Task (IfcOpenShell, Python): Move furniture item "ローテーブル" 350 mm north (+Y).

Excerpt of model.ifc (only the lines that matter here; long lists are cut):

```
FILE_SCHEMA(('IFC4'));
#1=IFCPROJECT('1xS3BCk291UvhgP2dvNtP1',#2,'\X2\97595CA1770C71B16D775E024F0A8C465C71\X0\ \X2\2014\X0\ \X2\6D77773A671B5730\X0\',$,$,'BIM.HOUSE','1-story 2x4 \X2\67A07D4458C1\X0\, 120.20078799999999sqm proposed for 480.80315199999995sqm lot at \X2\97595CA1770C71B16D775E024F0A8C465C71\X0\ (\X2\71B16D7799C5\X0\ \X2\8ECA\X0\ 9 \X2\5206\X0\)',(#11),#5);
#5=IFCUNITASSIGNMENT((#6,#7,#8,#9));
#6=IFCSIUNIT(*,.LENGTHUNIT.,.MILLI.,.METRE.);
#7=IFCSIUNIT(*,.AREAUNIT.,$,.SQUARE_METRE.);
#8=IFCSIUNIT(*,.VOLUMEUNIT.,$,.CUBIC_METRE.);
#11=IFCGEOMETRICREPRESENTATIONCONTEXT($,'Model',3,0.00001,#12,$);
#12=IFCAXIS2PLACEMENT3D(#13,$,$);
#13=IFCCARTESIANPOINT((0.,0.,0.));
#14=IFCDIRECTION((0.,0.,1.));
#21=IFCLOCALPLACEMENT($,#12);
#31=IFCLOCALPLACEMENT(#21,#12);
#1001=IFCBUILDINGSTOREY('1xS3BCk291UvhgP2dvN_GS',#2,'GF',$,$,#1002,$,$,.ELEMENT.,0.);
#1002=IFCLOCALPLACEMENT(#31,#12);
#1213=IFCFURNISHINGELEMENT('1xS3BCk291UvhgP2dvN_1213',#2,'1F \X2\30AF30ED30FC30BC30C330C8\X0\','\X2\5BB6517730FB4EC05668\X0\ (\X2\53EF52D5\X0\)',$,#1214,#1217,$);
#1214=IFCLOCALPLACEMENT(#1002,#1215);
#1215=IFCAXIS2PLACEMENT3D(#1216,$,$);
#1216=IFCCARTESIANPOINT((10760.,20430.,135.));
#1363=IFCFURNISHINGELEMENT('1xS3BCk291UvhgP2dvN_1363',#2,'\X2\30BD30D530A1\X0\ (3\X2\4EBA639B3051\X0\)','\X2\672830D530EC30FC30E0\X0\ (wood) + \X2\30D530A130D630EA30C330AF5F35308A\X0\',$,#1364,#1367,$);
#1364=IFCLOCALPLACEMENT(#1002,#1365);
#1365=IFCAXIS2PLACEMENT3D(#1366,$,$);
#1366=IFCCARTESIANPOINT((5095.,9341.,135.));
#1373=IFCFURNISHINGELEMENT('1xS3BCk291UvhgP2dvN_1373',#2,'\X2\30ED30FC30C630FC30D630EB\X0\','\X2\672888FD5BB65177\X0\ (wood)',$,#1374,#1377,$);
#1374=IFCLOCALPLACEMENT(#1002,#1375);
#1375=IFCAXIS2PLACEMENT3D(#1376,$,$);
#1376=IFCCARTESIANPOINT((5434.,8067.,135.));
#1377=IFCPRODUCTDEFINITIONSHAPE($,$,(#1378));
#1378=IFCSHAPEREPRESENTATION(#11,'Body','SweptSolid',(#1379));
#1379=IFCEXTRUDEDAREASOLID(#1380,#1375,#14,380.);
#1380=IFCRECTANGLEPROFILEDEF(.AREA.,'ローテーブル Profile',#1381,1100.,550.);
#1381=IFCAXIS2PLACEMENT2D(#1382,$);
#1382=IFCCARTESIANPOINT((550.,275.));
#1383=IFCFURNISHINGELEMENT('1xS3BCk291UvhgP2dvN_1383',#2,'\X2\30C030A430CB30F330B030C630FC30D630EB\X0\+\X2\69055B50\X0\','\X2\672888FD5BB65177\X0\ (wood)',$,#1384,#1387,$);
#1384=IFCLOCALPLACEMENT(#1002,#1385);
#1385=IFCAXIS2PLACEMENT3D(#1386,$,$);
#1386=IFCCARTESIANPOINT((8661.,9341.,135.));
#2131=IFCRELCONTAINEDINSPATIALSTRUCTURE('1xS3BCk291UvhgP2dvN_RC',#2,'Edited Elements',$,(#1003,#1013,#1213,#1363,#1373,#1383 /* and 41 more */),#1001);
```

```python
import ifcopenshell
import ifcopenshell.api.geometry
import ifcopenshell.util.placement
import ifcopenshell.util.unit

model = ifcopenshell.open("model.ifc")
unit_scale = ifcopenshell.util.unit.calculate_unit_scale(model)

item = model.by_id(1373)
matrix = ifcopenshell.util.placement.get_local_placement(item.ObjectPlacement)
matrix[1, 3] += 0.35 / unit_scale
ifcopenshell.api.geometry.edit_object_placement(model, product=item, matrix=matrix, is_si=False)

print(ifcopenshell.util.placement.get_local_placement(item.ObjectPlacement).round(3) + 0.0)

model.write("model_v2.ifc")
```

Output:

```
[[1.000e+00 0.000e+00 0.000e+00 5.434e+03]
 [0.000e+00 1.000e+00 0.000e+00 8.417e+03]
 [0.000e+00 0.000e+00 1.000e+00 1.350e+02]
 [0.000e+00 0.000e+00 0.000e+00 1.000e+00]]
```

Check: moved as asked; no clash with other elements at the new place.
